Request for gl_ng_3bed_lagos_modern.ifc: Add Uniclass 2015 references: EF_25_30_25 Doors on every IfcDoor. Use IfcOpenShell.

First a look at what the model holds.

```python
import ifcopenshell

model = ifcopenshell.open("gl_ng_3bed_lagos_modern.ifc")
print(model.schema)
print("classifications:", [c.Name for c in model.by_type("IfcClassification")])
for ifc_class in ("IfcDoor", "IfcRoof", "IfcStair", "IfcWall", "IfcWindow"):
    print(ifc_class, len(model.by_type(ifc_class)))
```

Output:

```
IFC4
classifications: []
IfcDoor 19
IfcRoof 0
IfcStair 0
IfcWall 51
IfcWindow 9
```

```python
import ifcopenshell
import ifcopenshell.api.classification

model = ifcopenshell.open("gl_ng_3bed_lagos_modern.ifc")

system = ifcopenshell.api.classification.add_classification(model, classification="Uniclass 2015")

codes = {
    "IfcDoor": ("EF_25_30_25", "Doors"),
}
for ifc_class, (code, name) in codes.items():
    products = model.by_type(ifc_class)
    ifcopenshell.api.classification.add_reference(
        model, products=products, classification=system, identification=code, name=name
    )
    print(code, len(products))

model.write("gl_ng_3bed_lagos_modern_updated.ifc")
```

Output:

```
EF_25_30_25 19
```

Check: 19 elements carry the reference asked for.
